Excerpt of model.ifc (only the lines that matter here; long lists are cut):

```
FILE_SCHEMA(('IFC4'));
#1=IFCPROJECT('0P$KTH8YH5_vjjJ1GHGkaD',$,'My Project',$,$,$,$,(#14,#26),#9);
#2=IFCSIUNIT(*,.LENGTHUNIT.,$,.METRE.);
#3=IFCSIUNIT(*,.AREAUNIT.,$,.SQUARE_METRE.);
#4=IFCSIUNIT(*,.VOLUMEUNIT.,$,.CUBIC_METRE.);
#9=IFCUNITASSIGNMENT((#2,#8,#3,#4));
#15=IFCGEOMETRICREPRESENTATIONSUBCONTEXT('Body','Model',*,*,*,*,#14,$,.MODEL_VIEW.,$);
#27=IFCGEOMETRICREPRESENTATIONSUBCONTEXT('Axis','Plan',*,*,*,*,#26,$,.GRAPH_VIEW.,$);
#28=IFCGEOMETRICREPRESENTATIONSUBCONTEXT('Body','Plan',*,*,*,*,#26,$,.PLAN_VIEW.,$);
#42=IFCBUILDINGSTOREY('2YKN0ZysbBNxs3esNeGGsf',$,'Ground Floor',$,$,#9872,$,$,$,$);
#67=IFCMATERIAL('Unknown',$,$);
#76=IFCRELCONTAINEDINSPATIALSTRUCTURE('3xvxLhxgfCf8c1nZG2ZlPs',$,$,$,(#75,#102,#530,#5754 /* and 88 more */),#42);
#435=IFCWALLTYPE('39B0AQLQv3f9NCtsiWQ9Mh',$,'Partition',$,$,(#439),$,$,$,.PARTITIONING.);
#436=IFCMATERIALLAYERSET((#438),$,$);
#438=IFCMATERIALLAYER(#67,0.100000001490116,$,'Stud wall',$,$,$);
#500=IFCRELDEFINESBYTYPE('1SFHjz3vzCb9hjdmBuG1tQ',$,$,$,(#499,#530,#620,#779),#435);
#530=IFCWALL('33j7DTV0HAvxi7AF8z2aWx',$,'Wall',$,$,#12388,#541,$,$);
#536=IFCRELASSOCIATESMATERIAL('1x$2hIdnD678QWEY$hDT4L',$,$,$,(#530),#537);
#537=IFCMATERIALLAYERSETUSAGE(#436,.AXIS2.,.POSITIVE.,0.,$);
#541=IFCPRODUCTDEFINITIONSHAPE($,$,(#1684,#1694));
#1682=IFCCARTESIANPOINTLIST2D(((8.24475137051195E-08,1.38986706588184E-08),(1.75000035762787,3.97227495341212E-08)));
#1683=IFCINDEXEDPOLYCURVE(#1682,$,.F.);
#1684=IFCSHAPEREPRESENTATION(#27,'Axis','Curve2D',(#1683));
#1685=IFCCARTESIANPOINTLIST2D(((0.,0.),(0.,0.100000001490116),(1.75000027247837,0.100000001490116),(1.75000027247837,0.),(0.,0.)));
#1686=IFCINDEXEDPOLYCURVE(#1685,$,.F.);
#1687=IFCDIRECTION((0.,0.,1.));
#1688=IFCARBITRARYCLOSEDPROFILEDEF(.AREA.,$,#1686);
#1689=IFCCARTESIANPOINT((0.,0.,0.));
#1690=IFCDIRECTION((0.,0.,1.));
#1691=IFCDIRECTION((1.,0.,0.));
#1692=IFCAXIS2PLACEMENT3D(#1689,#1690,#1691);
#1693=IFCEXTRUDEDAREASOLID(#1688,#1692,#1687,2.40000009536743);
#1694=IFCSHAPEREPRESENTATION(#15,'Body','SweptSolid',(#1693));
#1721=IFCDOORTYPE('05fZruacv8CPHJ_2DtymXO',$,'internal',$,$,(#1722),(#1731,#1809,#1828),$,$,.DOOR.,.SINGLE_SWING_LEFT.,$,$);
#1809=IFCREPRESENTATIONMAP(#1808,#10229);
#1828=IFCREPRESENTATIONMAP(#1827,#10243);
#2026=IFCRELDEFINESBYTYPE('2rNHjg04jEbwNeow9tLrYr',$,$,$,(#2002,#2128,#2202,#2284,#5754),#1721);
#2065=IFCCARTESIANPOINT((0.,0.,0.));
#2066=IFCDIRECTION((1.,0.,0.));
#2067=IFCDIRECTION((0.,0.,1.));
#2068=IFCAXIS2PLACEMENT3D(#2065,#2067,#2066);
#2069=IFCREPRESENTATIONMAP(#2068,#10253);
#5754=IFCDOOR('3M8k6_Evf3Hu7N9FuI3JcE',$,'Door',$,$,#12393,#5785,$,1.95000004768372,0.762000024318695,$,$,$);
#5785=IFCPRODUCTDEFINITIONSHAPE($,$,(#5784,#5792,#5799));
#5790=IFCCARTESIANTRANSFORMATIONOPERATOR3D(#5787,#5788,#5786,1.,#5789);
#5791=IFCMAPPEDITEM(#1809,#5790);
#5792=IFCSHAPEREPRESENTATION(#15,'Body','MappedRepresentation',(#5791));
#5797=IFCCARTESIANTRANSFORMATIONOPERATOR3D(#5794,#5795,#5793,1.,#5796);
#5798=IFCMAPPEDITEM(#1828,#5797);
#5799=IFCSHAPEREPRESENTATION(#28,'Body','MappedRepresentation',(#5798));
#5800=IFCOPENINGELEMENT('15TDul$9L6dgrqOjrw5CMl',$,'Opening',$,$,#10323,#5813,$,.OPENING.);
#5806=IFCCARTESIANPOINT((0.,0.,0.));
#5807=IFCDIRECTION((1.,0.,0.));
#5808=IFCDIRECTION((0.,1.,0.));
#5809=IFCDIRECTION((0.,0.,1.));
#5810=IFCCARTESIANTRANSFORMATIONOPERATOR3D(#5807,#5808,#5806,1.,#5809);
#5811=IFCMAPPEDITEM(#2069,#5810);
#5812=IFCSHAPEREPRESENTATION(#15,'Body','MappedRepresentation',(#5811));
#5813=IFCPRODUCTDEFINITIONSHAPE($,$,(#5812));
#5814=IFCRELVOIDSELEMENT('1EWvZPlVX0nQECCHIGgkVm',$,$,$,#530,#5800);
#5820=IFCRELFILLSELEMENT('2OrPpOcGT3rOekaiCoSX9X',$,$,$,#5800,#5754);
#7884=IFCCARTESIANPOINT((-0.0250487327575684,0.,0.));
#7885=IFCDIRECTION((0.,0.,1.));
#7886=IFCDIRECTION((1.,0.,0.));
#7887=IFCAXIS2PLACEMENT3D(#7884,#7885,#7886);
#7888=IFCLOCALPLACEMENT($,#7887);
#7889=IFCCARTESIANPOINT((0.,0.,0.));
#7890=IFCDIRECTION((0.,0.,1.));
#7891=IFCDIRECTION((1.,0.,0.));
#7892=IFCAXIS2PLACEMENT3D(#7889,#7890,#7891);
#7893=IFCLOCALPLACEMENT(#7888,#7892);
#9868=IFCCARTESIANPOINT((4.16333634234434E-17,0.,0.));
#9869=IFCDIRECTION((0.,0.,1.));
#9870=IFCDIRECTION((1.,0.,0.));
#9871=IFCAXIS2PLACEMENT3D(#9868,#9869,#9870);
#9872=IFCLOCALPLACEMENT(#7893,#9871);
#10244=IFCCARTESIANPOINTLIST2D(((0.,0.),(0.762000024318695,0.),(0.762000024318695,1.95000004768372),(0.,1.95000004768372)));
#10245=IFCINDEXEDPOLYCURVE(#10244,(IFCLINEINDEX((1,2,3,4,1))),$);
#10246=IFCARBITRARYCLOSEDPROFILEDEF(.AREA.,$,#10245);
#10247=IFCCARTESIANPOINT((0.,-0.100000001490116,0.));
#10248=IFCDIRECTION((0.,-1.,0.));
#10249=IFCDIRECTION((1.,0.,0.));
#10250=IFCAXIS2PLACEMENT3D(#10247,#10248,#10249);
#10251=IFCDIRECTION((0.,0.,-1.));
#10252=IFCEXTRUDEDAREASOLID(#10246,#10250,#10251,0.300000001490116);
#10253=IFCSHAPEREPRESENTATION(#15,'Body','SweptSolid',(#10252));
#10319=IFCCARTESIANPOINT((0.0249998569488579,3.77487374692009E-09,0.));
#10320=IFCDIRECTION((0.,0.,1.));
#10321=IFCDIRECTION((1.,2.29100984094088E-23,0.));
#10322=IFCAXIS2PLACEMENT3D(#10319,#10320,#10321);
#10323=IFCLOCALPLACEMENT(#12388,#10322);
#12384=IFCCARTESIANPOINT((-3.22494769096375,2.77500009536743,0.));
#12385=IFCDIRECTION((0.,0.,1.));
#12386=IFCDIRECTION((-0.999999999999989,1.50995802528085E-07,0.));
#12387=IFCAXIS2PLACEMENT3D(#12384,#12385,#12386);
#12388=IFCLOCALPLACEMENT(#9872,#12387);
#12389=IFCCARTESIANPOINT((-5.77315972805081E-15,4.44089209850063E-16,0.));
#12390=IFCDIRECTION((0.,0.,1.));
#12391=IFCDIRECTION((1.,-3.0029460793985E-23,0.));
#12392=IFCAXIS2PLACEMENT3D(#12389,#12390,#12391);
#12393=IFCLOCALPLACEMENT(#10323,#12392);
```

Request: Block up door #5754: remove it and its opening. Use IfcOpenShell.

```python
import ifcopenshell
import ifcopenshell.api.feature
import ifcopenshell.api.root
import ifcopenshell.geom
import ifcopenshell.util.shape

model = ifcopenshell.open("model.ifc")
settings = ifcopenshell.geom.settings()


def volume(element):
    """Net volume in cubic metres, openings subtracted."""
    shape = ifcopenshell.geom.create_shape(settings, element)
    return ifcopenshell.util.shape.get_volume(shape.geometry)


door = model.by_guid("3M8k6_Evf3Hu7N9FuI3JcE")
opening = door.FillsVoids[0].RelatingOpeningElement
wall = opening.VoidsElements[0].RelatingBuildingElement
before = volume(wall)

ifcopenshell.api.root.remove_product(model, product=door)
ifcopenshell.api.feature.remove_feature(model, feature=opening)

after = volume(wall)

print(f"wall volume {before:.3f} -> {after:.3f} m3")

model.write("model_edited.ifc")
```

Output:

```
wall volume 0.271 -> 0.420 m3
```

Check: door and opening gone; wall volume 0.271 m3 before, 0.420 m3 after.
